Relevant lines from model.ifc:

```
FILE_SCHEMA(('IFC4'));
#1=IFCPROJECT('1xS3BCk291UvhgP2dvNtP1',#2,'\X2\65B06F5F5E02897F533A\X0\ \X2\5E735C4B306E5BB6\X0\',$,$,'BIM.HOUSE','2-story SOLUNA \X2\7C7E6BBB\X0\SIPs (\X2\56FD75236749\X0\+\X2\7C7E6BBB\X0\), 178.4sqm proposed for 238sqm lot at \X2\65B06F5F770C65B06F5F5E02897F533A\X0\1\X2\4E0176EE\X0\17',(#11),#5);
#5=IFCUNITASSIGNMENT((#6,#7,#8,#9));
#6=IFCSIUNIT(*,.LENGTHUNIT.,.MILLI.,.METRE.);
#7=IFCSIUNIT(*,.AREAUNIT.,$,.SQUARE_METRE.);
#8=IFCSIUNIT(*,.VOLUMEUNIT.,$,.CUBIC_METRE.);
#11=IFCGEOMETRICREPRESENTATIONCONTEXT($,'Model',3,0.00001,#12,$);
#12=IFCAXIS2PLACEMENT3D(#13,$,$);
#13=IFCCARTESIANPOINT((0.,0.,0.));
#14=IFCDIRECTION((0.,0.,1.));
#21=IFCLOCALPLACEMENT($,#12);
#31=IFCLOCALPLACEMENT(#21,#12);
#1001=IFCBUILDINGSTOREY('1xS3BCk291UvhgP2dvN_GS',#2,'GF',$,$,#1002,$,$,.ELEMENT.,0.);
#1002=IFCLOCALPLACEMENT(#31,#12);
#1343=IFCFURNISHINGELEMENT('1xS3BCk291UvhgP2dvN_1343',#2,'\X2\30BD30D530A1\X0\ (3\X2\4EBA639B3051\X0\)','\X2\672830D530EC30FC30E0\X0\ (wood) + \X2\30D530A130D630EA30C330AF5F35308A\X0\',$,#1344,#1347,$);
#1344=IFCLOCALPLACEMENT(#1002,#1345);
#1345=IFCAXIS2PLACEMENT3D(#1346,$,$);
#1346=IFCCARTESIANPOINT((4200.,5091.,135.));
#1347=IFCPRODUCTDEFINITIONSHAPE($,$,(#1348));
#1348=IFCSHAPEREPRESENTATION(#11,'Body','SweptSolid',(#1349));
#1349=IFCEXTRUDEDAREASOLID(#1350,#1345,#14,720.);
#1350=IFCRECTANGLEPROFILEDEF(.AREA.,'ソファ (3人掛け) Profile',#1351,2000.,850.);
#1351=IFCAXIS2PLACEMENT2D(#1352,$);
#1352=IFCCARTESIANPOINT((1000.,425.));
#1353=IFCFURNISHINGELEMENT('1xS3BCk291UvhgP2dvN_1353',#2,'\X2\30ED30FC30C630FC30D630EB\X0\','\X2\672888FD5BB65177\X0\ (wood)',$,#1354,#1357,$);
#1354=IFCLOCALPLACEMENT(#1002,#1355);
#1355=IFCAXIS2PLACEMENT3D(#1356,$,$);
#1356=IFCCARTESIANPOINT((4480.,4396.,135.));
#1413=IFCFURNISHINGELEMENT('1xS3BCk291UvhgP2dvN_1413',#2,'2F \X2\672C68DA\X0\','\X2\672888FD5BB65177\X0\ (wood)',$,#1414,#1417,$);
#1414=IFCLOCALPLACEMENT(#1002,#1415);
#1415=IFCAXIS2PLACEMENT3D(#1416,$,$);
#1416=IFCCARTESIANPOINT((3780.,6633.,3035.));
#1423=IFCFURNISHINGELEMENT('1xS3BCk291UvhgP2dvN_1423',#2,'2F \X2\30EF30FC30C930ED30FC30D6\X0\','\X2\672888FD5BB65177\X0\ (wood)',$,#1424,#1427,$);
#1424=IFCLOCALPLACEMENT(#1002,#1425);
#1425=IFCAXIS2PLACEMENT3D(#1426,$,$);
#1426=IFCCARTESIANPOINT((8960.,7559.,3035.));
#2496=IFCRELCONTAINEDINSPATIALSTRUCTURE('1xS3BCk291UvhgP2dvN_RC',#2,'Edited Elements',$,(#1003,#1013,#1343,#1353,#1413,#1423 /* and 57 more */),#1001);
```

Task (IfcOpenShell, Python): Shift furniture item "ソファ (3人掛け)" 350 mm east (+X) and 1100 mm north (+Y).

```python
import ifcopenshell
import ifcopenshell.api.geometry
import ifcopenshell.util.placement

model = ifcopenshell.open("model.ifc")

item = model.by_id(1343)
matrix = ifcopenshell.util.placement.get_local_placement(item.ObjectPlacement)
matrix[0, 3] += 350.0
matrix[1, 3] += 1100.0
ifcopenshell.api.geometry.edit_object_placement(model, product=item, matrix=matrix, is_si=False)

print(ifcopenshell.util.placement.get_local_placement(item.ObjectPlacement).round(3) + 0.0)

model.write("model_rev.ifc")
```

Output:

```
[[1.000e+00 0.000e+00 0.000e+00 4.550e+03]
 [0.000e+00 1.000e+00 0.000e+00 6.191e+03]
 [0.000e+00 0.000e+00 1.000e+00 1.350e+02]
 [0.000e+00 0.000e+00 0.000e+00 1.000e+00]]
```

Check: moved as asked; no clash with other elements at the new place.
